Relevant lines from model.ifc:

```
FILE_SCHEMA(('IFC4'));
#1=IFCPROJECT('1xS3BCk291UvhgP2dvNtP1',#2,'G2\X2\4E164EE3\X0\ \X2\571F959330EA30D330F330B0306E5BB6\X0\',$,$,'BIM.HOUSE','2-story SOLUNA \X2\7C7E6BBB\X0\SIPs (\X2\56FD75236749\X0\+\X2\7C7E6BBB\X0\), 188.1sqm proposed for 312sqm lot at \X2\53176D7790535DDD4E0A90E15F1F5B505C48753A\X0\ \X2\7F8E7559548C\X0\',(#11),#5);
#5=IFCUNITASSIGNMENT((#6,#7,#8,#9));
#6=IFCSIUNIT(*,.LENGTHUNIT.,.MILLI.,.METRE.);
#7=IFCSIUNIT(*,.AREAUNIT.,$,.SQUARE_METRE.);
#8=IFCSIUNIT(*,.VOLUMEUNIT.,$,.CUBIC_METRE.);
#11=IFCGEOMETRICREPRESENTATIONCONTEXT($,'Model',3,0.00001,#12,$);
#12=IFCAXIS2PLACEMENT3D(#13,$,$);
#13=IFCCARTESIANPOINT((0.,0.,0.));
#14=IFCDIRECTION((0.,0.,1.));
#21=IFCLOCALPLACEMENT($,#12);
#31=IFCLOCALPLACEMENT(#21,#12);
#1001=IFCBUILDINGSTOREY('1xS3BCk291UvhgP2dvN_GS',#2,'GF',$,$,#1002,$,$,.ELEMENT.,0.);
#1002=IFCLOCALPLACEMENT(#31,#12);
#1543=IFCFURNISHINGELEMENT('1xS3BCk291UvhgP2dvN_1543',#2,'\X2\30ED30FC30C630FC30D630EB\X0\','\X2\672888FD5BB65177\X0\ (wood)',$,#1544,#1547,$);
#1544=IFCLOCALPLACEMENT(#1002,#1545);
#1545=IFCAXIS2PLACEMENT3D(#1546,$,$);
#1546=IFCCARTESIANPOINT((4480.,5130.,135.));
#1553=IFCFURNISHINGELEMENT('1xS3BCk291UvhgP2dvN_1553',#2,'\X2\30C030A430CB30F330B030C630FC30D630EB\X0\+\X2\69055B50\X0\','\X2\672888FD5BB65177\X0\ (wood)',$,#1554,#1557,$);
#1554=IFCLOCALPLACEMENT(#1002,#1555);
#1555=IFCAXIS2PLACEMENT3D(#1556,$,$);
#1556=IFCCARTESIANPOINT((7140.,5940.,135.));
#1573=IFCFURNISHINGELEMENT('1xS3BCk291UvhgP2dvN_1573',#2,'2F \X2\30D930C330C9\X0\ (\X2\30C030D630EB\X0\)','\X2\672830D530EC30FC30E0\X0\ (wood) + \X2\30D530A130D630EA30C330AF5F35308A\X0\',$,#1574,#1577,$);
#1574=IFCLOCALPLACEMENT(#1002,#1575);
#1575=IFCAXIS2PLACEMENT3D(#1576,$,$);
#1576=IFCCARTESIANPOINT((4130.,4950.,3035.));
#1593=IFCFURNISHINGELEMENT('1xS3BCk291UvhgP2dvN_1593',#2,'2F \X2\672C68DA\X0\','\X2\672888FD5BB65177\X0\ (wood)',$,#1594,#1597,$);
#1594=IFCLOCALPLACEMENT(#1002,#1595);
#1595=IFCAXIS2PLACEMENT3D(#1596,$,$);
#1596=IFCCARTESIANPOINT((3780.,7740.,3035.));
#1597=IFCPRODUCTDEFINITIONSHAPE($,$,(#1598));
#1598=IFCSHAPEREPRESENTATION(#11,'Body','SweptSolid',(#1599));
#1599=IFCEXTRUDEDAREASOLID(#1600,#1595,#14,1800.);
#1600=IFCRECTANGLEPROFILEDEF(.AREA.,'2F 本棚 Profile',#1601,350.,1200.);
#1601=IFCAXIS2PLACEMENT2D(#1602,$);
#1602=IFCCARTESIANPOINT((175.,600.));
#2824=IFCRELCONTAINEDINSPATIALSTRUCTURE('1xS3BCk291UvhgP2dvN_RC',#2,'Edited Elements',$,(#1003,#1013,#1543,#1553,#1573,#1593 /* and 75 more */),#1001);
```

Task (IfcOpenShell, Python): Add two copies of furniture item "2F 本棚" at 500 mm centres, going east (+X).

```python
import numpy as np
import ifcopenshell
import ifcopenshell.api.geometry
import ifcopenshell.api.root
import ifcopenshell.util.element
import ifcopenshell.util.placement

model = ifcopenshell.open("model.ifc")


def reuse_history(source, copy):
    """copy_class also copies each property set's owner history, people and application; keep the originals."""
    for rel in copy.IsDefinedBy:
        if rel.is_a("IfcRelDefinesByProperties") and (history := rel.RelatingPropertyDefinition.OwnerHistory):
            rel.RelatingPropertyDefinition.OwnerHistory = source.OwnerHistory
            ifcopenshell.util.element.remove_deep2(model, history)


source = model.by_guid("1xS3BCk291UvhgP2dvN_1593")
base = ifcopenshell.util.placement.get_local_placement(source.ObjectPlacement)
step = np.array([1.0, 0.0, 0.0]) * 500.0

for i in range(1, 3):
    copy = ifcopenshell.api.root.copy_class(model, product=source)
    copy.Representation = ifcopenshell.util.element.copy_deep(
        model, source.Representation, exclude=["IfcGeometricRepresentationContext", "IfcRepresentationMap"]
    )
    reuse_history(source, copy)
    matrix = base.copy()
    matrix[:3, 3] += i * step
    print("added at", matrix[:3, 3].round(3) + 0.0)
    ifcopenshell.api.geometry.edit_object_placement(model, product=copy, matrix=matrix, is_si=False)

model.write("model_edited.ifc")
```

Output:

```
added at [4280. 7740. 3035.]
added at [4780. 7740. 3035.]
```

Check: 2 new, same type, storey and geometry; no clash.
